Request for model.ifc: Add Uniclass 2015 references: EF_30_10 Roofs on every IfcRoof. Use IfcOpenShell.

First a look at what the model holds.

```python
import ifcopenshell

model = ifcopenshell.open("model.ifc")
print(model.schema)
print("classifications:", [c.Name for c in model.by_type("IfcClassification")])
for ifc_class in ("IfcDoor", "IfcRoof", "IfcStair", "IfcWall", "IfcWindow"):
    print(ifc_class, len(model.by_type(ifc_class)))
```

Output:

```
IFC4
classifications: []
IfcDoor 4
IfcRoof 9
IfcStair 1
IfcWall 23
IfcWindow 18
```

```python
import ifcopenshell
import ifcopenshell.api.classification

model = ifcopenshell.open("model.ifc")

system = ifcopenshell.api.classification.add_classification(model, classification="Uniclass 2015")

codes = {
    "IfcRoof": ("EF_30_10", "Roofs"),
}
for ifc_class, (code, name) in codes.items():
    products = model.by_type(ifc_class)
    ifcopenshell.api.classification.add_reference(
        model, products=products, classification=system, identification=code, name=name
    )
    print(code, len(products))

model.write("model_updated.ifc")
```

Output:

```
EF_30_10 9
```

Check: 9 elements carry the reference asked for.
